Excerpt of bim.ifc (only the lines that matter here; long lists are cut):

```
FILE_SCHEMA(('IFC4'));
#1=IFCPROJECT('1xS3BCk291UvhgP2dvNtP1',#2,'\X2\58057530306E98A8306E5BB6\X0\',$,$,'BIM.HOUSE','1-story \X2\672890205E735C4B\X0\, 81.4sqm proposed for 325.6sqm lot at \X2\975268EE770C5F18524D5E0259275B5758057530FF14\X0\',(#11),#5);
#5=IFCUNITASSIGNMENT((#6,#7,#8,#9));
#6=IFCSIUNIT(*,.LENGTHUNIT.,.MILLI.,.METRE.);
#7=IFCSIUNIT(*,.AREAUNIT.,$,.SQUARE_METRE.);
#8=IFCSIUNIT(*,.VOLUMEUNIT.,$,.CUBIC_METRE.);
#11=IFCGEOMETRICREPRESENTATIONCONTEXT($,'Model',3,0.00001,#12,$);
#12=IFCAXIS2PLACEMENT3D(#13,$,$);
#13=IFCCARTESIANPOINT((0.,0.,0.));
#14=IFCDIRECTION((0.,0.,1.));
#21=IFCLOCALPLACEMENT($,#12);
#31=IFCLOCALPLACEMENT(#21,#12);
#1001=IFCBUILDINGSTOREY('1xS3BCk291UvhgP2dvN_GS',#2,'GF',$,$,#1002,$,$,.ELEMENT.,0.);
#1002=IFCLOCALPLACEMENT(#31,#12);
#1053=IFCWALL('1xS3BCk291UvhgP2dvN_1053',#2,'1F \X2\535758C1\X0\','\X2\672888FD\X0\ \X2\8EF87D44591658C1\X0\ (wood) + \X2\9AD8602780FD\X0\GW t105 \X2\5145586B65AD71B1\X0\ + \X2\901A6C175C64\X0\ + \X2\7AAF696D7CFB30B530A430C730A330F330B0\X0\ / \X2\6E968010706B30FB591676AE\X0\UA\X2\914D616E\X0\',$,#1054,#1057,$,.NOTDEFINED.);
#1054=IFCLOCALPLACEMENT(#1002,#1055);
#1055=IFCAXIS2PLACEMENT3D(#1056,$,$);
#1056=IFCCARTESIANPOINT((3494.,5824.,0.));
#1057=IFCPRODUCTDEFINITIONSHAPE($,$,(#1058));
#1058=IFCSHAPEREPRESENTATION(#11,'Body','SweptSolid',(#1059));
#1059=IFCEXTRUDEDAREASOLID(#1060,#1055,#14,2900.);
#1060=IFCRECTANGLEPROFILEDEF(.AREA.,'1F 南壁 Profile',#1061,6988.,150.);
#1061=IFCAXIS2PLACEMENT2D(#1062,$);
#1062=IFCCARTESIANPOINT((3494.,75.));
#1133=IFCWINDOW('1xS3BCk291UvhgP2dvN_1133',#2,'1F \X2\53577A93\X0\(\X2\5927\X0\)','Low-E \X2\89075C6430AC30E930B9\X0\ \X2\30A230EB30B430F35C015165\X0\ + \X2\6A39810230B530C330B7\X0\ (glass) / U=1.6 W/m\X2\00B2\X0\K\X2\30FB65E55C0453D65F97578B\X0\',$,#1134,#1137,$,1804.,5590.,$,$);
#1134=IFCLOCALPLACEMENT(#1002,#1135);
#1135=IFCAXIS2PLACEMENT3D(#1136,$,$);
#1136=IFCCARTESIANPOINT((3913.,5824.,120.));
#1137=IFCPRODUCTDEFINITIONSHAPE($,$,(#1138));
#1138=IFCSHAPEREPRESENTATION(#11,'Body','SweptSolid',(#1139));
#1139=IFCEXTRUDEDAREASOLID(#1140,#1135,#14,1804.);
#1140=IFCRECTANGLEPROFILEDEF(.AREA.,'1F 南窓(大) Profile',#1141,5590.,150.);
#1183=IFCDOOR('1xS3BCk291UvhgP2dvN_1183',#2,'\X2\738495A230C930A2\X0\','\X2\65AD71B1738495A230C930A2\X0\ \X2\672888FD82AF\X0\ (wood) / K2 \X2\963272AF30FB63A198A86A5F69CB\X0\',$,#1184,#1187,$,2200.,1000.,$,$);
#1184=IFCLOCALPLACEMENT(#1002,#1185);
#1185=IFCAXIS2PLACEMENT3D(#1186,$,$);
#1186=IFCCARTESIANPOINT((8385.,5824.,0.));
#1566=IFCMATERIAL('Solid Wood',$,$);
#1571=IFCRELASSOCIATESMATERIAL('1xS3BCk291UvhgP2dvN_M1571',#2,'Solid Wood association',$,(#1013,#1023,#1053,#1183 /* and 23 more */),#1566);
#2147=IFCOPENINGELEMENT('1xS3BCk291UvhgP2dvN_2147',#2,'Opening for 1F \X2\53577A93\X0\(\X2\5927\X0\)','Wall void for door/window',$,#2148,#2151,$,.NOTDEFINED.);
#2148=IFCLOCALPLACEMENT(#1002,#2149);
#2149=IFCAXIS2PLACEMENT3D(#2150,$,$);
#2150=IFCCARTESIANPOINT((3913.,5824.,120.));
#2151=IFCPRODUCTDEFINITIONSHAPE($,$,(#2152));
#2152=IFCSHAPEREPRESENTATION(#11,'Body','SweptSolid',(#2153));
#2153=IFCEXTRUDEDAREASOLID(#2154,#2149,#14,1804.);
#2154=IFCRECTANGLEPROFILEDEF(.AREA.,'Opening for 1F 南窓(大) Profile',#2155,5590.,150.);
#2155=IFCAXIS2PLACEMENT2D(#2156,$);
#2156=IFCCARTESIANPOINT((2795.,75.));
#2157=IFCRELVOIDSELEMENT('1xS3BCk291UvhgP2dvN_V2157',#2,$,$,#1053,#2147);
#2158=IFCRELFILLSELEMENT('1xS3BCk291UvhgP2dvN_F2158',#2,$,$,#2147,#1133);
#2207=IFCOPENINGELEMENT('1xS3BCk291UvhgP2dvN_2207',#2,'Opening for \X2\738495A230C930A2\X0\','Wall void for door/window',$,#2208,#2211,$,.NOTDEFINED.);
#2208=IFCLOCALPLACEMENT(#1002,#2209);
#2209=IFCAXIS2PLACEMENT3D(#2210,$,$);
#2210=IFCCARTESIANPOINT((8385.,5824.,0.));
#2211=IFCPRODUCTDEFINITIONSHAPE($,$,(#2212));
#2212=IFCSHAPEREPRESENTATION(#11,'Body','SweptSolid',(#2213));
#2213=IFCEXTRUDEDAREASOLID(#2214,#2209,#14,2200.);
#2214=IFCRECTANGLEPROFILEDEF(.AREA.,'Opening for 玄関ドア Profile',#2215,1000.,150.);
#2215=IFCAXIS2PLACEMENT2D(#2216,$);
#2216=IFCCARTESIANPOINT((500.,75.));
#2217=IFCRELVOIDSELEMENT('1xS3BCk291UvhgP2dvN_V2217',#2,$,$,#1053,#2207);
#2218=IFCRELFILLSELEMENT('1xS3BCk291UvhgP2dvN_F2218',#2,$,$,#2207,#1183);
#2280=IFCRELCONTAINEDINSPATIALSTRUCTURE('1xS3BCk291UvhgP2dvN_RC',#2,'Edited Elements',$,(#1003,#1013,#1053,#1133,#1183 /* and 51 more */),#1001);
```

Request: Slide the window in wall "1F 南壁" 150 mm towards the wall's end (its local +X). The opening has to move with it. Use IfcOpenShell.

```python
import ifcopenshell
import ifcopenshell.api.geometry
import ifcopenshell.util.placement
import ifcopenshell.util.unit

model = ifcopenshell.open("bim.ifc")
unit_scale = ifcopenshell.util.unit.calculate_unit_scale(model)

window = model.by_guid("1xS3BCk291UvhgP2dvN_1133")
opening = window.FillsVoids[0].RelatingOpeningElement
wall = opening.VoidsElements[0].RelatingBuildingElement

wall_matrix = ifcopenshell.util.placement.get_local_placement(wall.ObjectPlacement)
shift = wall_matrix[:3, 0] * 0.15 / unit_scale
before = ifcopenshell.util.placement.get_local_placement(window.ObjectPlacement)[:3, 3].copy()

# The window is not placed relative to its opening, so move both.
for product in (opening, window):
    matrix = ifcopenshell.util.placement.get_local_placement(product.ObjectPlacement)
    matrix[:3, 3] += shift
    ifcopenshell.api.geometry.edit_object_placement(model, product=product, matrix=matrix, is_si=False)

after = ifcopenshell.util.placement.get_local_placement(window.ObjectPlacement)[:3, 3]
print("window moved by", (after - before).round(3) + 0.0)

model.write("bim_edited.ifc")
```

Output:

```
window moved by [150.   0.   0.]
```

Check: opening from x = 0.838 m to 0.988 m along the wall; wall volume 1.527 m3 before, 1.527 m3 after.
